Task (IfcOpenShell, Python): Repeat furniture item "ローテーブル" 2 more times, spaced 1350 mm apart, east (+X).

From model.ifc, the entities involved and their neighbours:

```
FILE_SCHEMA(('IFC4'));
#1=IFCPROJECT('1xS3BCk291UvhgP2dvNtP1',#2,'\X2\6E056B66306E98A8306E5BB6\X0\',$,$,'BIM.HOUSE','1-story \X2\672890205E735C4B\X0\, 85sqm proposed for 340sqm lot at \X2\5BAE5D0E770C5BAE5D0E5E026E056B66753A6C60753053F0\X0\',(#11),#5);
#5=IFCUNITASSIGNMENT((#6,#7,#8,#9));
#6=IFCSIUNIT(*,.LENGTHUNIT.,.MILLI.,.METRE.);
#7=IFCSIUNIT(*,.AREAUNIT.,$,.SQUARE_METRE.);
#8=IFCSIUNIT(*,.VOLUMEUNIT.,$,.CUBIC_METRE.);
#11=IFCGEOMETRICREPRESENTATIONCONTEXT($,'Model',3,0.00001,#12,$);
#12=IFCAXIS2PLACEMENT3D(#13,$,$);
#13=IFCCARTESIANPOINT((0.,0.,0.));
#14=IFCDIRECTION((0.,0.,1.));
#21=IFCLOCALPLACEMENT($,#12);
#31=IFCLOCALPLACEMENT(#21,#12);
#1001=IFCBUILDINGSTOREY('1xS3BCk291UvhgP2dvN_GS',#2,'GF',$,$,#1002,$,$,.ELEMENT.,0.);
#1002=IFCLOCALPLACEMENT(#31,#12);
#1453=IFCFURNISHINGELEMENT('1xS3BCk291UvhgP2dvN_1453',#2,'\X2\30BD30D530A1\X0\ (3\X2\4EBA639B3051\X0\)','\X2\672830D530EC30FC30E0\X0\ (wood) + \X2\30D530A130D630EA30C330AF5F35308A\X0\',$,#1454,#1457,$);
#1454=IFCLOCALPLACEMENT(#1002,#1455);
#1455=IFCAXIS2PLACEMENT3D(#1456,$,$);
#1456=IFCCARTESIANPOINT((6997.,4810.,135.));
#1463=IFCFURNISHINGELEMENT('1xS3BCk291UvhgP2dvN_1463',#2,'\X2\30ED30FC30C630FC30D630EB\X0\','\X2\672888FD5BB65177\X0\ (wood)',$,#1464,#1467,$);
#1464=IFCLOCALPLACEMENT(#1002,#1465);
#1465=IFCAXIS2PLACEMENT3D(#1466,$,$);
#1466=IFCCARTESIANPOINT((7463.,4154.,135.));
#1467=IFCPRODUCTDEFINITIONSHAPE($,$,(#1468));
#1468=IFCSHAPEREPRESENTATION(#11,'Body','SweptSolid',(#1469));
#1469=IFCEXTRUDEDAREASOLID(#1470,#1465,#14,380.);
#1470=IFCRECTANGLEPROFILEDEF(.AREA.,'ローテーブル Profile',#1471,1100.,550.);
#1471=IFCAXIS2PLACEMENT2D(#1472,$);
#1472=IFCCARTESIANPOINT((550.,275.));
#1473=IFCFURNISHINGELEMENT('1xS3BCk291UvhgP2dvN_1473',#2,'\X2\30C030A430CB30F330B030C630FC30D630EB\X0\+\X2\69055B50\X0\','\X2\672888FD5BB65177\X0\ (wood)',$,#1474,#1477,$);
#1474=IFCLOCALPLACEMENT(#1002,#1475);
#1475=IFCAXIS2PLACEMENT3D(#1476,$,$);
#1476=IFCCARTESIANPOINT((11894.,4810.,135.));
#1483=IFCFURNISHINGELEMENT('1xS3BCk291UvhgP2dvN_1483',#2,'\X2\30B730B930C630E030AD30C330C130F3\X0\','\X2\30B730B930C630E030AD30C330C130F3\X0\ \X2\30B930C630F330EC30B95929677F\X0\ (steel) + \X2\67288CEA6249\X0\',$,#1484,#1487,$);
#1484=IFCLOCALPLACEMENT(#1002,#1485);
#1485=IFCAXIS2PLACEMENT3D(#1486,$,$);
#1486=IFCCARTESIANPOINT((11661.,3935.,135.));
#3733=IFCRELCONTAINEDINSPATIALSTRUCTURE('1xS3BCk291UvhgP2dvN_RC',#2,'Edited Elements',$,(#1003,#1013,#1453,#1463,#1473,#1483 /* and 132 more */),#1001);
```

```python
import numpy as np
import ifcopenshell
import ifcopenshell.api.geometry
import ifcopenshell.api.root
import ifcopenshell.util.element
import ifcopenshell.util.placement
import ifcopenshell.util.unit

model = ifcopenshell.open("model.ifc")
unit_scale = ifcopenshell.util.unit.calculate_unit_scale(model)


def reuse_history(source, copy):
    """copy_class also copies each property set's owner history, people and application; keep the originals."""
    for rel in copy.IsDefinedBy:
        if rel.is_a("IfcRelDefinesByProperties") and (history := rel.RelatingPropertyDefinition.OwnerHistory):
            rel.RelatingPropertyDefinition.OwnerHistory = source.OwnerHistory
            ifcopenshell.util.element.remove_deep2(model, history)


source = model.by_guid("1xS3BCk291UvhgP2dvN_1463")
base = ifcopenshell.util.placement.get_local_placement(source.ObjectPlacement)
step = np.array([1.0, 0.0, 0.0]) * 1.35 / unit_scale

for i in range(1, 3):
    copy = ifcopenshell.api.root.copy_class(model, product=source)
    copy.Representation = ifcopenshell.util.element.copy_deep(
        model, source.Representation, exclude=["IfcGeometricRepresentationContext", "IfcRepresentationMap"]
    )
    reuse_history(source, copy)
    matrix = base.copy()
    matrix[:3, 3] += i * step
    print("added at", matrix[:3, 3].round(3) + 0.0)
    ifcopenshell.api.geometry.edit_object_placement(model, product=copy, matrix=matrix, is_si=False)

model.write("model-out.ifc")
```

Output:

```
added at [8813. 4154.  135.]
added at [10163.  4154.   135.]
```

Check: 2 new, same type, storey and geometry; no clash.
